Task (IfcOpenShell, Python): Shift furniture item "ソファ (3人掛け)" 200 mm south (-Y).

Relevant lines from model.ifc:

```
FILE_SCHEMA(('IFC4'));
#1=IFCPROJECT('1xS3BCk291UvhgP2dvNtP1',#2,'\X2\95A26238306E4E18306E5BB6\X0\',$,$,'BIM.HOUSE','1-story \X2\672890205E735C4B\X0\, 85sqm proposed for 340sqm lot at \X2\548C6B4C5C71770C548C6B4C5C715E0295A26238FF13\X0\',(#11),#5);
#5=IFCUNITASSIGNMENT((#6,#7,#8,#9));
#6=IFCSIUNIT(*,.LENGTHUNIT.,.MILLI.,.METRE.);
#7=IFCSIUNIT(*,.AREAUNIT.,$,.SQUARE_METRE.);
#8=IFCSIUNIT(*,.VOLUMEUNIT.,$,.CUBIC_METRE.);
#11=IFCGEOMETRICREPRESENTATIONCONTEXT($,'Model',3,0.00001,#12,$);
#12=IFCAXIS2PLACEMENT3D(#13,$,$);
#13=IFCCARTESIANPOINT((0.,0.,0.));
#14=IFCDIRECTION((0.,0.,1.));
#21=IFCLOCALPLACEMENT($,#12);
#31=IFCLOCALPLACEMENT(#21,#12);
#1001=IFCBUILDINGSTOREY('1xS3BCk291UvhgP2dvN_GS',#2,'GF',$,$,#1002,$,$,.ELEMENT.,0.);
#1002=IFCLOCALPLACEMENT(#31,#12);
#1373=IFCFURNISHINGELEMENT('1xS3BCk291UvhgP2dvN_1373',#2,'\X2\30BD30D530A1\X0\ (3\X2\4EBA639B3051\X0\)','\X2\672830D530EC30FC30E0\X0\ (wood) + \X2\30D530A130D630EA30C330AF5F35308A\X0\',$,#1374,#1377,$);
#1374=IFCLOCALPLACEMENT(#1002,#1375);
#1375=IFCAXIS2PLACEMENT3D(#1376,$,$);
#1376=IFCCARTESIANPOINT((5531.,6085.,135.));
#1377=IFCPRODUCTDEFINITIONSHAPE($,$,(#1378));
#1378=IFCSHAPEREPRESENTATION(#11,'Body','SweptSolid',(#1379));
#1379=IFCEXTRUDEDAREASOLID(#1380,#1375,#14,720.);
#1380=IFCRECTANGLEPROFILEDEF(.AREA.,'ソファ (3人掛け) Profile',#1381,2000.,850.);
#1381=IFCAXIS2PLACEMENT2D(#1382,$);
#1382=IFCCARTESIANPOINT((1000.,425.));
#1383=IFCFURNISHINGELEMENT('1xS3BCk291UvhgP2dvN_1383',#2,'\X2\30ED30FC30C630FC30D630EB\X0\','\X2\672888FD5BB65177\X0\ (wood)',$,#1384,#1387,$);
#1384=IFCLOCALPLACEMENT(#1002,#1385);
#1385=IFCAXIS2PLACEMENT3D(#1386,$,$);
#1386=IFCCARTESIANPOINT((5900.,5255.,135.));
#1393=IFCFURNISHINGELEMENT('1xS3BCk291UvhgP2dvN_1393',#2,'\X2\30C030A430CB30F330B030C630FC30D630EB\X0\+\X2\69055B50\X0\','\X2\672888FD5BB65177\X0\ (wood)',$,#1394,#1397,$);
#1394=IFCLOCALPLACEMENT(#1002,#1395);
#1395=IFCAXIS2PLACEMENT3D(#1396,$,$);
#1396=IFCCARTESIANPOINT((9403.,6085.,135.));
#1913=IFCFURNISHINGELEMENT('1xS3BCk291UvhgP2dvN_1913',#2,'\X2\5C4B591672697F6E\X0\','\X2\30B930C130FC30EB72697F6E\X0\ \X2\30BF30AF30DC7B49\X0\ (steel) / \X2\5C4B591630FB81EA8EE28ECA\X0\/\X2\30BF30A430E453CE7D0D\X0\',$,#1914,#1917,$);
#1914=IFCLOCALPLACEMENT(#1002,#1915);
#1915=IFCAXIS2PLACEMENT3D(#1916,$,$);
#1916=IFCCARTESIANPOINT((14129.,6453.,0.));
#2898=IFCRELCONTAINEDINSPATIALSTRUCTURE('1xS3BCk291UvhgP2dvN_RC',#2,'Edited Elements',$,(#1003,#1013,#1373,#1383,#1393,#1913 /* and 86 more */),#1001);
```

```python
import ifcopenshell
import ifcopenshell.api.geometry
import ifcopenshell.util.placement
import ifcopenshell.util.unit

model = ifcopenshell.open("model.ifc")
unit_scale = ifcopenshell.util.unit.calculate_unit_scale(model)

item = model.by_id(1373)
matrix = ifcopenshell.util.placement.get_local_placement(item.ObjectPlacement)
matrix[1, 3] -= 0.2 / unit_scale
ifcopenshell.api.geometry.edit_object_placement(model, product=item, matrix=matrix, is_si=False)

print(ifcopenshell.util.placement.get_local_placement(item.ObjectPlacement).round(3) + 0.0)

model.write("model_v2.ifc")
```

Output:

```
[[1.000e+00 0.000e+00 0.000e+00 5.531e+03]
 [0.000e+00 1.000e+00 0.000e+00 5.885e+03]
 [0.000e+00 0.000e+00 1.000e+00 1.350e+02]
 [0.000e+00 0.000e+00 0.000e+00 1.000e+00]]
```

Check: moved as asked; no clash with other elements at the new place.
